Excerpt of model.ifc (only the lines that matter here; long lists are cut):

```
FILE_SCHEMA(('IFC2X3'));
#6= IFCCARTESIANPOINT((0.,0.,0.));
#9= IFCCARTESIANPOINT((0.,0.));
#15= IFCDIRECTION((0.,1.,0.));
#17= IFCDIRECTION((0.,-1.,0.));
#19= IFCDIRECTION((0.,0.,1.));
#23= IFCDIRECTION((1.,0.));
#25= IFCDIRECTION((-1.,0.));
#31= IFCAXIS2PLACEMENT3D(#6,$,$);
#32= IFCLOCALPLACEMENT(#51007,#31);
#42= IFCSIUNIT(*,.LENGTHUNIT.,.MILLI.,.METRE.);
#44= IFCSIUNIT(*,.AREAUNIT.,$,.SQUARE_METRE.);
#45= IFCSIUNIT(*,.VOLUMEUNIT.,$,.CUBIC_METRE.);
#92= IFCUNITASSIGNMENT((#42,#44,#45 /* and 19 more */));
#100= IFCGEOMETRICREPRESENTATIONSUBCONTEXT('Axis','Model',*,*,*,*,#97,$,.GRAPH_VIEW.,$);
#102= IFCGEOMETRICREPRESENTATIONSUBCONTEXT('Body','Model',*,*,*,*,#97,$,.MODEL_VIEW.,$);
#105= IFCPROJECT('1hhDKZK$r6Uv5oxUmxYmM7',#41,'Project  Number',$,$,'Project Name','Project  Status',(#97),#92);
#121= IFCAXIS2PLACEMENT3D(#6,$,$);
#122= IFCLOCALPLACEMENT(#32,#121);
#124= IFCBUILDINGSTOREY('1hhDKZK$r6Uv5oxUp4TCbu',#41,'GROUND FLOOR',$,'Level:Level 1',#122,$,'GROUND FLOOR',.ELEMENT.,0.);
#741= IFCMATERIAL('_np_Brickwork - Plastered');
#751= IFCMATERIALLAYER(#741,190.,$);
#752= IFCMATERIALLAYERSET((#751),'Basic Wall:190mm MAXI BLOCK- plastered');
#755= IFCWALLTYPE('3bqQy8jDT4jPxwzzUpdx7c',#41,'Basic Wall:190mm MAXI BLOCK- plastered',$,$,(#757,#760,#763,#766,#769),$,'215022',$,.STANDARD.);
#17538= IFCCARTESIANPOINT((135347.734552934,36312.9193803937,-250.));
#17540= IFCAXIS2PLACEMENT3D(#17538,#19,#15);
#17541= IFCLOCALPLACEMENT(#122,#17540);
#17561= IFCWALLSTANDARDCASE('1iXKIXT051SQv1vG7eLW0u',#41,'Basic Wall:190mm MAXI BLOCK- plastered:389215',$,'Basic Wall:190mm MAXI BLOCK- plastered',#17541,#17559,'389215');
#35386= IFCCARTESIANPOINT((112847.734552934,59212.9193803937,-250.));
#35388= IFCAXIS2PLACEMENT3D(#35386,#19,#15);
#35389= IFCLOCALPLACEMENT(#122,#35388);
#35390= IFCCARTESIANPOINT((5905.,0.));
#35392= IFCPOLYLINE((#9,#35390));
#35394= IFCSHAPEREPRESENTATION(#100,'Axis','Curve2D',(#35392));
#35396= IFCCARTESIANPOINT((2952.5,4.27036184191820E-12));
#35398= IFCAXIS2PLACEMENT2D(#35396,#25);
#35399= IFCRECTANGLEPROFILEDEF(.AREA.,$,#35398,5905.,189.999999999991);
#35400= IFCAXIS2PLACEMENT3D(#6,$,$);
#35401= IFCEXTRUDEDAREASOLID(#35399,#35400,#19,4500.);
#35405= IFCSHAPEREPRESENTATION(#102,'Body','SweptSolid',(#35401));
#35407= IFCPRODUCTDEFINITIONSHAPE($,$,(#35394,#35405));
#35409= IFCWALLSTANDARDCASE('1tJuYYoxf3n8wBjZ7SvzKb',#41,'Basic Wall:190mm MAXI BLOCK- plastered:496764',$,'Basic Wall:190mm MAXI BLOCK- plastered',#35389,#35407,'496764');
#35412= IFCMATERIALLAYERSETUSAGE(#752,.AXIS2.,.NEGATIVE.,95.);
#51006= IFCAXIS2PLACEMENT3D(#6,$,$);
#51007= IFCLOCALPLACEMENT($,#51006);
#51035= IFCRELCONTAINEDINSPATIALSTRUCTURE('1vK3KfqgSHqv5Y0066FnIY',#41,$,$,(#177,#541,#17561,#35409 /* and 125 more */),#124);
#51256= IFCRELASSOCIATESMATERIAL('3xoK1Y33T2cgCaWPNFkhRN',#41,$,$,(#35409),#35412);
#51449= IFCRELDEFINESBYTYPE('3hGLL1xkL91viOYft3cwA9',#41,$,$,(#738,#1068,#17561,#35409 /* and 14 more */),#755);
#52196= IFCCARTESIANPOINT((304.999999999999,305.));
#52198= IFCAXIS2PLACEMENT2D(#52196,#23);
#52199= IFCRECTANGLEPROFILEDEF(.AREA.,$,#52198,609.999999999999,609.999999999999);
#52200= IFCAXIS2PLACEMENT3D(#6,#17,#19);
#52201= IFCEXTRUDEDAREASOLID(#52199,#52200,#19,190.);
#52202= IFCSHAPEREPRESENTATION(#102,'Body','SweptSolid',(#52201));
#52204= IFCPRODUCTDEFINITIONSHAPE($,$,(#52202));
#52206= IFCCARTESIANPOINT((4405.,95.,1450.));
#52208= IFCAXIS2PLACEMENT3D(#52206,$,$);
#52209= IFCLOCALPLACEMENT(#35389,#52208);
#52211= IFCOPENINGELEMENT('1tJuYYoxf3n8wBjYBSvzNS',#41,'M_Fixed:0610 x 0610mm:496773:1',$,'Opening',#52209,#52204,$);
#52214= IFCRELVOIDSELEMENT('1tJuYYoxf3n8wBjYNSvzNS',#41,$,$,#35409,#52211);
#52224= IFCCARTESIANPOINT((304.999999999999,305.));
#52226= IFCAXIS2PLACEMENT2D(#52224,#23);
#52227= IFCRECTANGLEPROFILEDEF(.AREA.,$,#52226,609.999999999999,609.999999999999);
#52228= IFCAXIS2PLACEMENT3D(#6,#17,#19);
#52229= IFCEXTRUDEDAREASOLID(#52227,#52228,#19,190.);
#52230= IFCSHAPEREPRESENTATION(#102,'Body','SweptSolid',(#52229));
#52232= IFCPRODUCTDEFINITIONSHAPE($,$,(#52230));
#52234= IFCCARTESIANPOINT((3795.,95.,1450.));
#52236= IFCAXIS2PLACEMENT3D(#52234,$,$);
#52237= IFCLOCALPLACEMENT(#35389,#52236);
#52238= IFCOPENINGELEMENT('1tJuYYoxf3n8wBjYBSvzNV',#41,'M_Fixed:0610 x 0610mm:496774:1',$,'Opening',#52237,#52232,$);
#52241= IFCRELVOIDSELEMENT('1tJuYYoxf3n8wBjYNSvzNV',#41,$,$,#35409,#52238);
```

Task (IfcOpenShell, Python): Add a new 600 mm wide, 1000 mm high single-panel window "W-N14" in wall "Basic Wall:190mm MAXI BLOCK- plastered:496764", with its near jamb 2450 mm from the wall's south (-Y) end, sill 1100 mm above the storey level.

```python
import numpy as np
import ifcopenshell
import ifcopenshell.api.feature
import ifcopenshell.api.geometry
import ifcopenshell.api.root
import ifcopenshell.api.spatial
import ifcopenshell.api.type
import ifcopenshell.geom
import ifcopenshell.util.element
import ifcopenshell.util.placement
import ifcopenshell.util.representation
import ifcopenshell.util.shape
import ifcopenshell.util.unit

model = ifcopenshell.open("model.ifc")
unit_scale = ifcopenshell.util.unit.calculate_unit_scale(model)
settings = ifcopenshell.geom.settings()


def volume(element):
    """Net volume in cubic metres, openings subtracted."""
    shape = ifcopenshell.geom.create_shape(settings, element)
    return ifcopenshell.util.shape.get_volume(shape.geometry)


wall = model.by_id(35409)
storey = ifcopenshell.util.element.get_container(wall, ifc_class="IfcBuildingStorey")
context = ifcopenshell.util.representation.get_context(model, "Model", "Body", "MODEL_VIEW")
before = volume(wall)

width, height, from_end, sill = 0.6, 1, 2.45, 1.1  # metres

# The wall runs along its own X axis, and the end named is its -X end.
wall_shape = ifcopenshell.geom.create_shape(settings, wall)
x, y, z = ifcopenshell.util.shape.get_vertices(wall_shape.geometry).T
start = x.min() + from_end
face, thickness = float(y.min()), float(y.max() - y.min())
wall_matrix = ifcopenshell.util.placement.get_local_placement(wall.ObjectPlacement)
level = ifcopenshell.util.placement.get_local_placement(storey.ObjectPlacement)[2, 3]


def in_wall(x, y):
    """Placement at x, y metres in the wall's axes, at sill height."""
    matrix = wall_matrix.copy()
    matrix[:, 3] = wall_matrix @ np.array([x / unit_scale, y / unit_scale, 0.0, 1.0])
    matrix[2, 3] = level + sill / unit_scale
    return matrix


# Opening: a box that overshoots both wall faces by 50 mm.
opening = ifcopenshell.api.root.create_entity(model, ifc_class="IfcOpeningElement")
box = ifcopenshell.api.geometry.add_wall_representation(
    model, context=context, length=width, height=height, thickness=thickness + 0.1
)
ifcopenshell.api.geometry.assign_representation(model, product=opening, representation=box)
ifcopenshell.api.geometry.edit_object_placement(model, product=opening, matrix=in_wall(start, face - 0.05), is_si=False)
ifcopenshell.api.feature.add_feature(model, feature=opening, element=wall)

window = ifcopenshell.api.root.create_entity(model, ifc_class="IfcWindow", name="W-N14")
window.OverallWidth, window.OverallHeight = width / unit_scale, height / unit_scale
body = ifcopenshell.api.geometry.add_window_representation(
    model,
    context=context,
    overall_width=window.OverallWidth,
    overall_height=window.OverallHeight,
    partition_type="SINGLE_PANEL",
)
ifcopenshell.api.geometry.assign_representation(model, product=window, representation=body)
ifcopenshell.api.spatial.assign_container(model, products=[window], relating_structure=storey)
fills = ifcopenshell.api.feature.add_filling(model, opening=opening, element=window)
fills.OwnerHistory = window.OwnerHistory  # required in IFC2X3

# IFC2X3 keeps the operation on the window style.
style = ifcopenshell.api.root.create_entity(model, ifc_class="IfcWindowStyle", name="W-N14")
style.OperationType, style.ConstructionType = "SINGLE_PANEL", "NOTDEFINED"
style.ParameterTakesPrecedence = style.Sizeable = False
ifcopenshell.api.type.assign_type(model, related_objects=[window], relating_type=style)

# Centre the window in the wall's thickness.
ifcopenshell.api.geometry.edit_object_placement(model, product=window, matrix=in_wall(start, face), is_si=False)
window_shape = ifcopenshell.geom.create_shape(settings, window)
depth = ifcopenshell.util.shape.get_vertices(window_shape.geometry)[:, 1]
offset = face + thickness / 2 - (depth.min() + depth.max()) / 2
ifcopenshell.api.geometry.edit_object_placement(model, product=window, matrix=in_wall(start, offset), is_si=False)

after = volume(wall)

print(f"wall volume {before:.3f} -> {after:.3f} m3")

model.write("model_rev.ifc")
```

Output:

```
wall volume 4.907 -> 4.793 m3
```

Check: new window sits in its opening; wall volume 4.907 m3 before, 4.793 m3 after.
